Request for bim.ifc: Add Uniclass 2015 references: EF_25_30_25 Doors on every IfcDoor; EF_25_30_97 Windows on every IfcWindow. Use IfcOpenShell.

First a look at what the model holds.

```python
import ifcopenshell

model = ifcopenshell.open("bim.ifc")
print(model.schema)
print("classifications:", [c.Name for c in model.by_type("IfcClassification")])
for ifc_class in ("IfcDoor", "IfcRoof", "IfcStair", "IfcWall", "IfcWindow"):
    print(ifc_class, len(model.by_type(ifc_class)))
```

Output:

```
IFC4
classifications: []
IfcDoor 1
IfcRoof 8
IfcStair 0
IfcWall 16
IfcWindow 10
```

```python
import ifcopenshell
import ifcopenshell.api.classification

model = ifcopenshell.open("bim.ifc")

system = ifcopenshell.api.classification.add_classification(model, classification="Uniclass 2015")

codes = {
    "IfcDoor": ("EF_25_30_25", "Doors"),
    "IfcWindow": ("EF_25_30_97", "Windows"),
}
for ifc_class, (code, name) in codes.items():
    products = model.by_type(ifc_class)
    ifcopenshell.api.classification.add_reference(
        model, products=products, classification=system, identification=code, name=name
    )
    print(code, len(products))

model.write("bim_updated.ifc")
```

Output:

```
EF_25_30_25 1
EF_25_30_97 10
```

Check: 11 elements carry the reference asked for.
